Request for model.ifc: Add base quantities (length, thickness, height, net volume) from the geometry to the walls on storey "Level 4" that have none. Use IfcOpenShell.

First a look at what the model holds.

```python
import ifcopenshell
import ifcopenshell.util.element
import ifcopenshell.util.unit

model = ifcopenshell.open("model.ifc")
print(model.schema)
for unit_type in ("LENGTHUNIT", "AREAUNIT", "VOLUMEUNIT"):
    print(unit_type, ifcopenshell.util.unit.calculate_unit_scale(model, unit_type))
storey = next(s for s in model.by_type("IfcBuildingStorey") if s.Name == "Level 4")
walls = [e for e in ifcopenshell.util.element.get_decomposition(storey) if e.is_a("IfcWall")]
for e in sorted(walls, key=lambda e: e.id()):
    print(e.id(), e.is_a(), e.Name, list(ifcopenshell.util.element.get_psets(e, qtos_only=True)), sep=" | ")
```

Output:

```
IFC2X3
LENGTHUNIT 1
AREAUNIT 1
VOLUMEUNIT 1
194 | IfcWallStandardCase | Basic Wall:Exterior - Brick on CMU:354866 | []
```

```python
import ifcopenshell
import ifcopenshell.api.pset
import ifcopenshell.geom
import ifcopenshell.util.element
import ifcopenshell.util.shape
import ifcopenshell.util.unit

model = ifcopenshell.open("model.ifc")
unit_scale = ifcopenshell.util.unit.calculate_unit_scale(model)
volume_scale = ifcopenshell.util.unit.calculate_unit_scale(model, "VOLUMEUNIT")
settings = ifcopenshell.geom.settings()

storey = next(s for s in model.by_type("IfcBuildingStorey") if s.Name == "Level 4")
walls = [e for e in ifcopenshell.util.element.get_decomposition(storey) if e.is_a("IfcWall")]

for e in sorted(walls, key=lambda e: e.id()):
    if ifcopenshell.util.element.get_psets(e, qtos_only=True, should_inherit=False):
        continue
    # Geometry comes back in metres, in the element's own axes.
    shape = ifcopenshell.geom.create_shape(settings, e)
    values = {
        "Length": ifcopenshell.util.shape.get_x(shape.geometry) / unit_scale,
        "Width": ifcopenshell.util.shape.get_y(shape.geometry) / unit_scale,
        "Height": ifcopenshell.util.shape.get_z(shape.geometry) / unit_scale,
        "NetVolume": ifcopenshell.util.shape.get_volume(shape.geometry) / volume_scale,
    }
    qto = ifcopenshell.api.pset.add_qto(model, product=e, name="BaseQuantities")
    ifcopenshell.api.pset.edit_qto(model, qto=qto, properties=values)
    print(e.id(), {k: round(v, 3) for k, v in values.items()})

model.write("model-out.ifc")
```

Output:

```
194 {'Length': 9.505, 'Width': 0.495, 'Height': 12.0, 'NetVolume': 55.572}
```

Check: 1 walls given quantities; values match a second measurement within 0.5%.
